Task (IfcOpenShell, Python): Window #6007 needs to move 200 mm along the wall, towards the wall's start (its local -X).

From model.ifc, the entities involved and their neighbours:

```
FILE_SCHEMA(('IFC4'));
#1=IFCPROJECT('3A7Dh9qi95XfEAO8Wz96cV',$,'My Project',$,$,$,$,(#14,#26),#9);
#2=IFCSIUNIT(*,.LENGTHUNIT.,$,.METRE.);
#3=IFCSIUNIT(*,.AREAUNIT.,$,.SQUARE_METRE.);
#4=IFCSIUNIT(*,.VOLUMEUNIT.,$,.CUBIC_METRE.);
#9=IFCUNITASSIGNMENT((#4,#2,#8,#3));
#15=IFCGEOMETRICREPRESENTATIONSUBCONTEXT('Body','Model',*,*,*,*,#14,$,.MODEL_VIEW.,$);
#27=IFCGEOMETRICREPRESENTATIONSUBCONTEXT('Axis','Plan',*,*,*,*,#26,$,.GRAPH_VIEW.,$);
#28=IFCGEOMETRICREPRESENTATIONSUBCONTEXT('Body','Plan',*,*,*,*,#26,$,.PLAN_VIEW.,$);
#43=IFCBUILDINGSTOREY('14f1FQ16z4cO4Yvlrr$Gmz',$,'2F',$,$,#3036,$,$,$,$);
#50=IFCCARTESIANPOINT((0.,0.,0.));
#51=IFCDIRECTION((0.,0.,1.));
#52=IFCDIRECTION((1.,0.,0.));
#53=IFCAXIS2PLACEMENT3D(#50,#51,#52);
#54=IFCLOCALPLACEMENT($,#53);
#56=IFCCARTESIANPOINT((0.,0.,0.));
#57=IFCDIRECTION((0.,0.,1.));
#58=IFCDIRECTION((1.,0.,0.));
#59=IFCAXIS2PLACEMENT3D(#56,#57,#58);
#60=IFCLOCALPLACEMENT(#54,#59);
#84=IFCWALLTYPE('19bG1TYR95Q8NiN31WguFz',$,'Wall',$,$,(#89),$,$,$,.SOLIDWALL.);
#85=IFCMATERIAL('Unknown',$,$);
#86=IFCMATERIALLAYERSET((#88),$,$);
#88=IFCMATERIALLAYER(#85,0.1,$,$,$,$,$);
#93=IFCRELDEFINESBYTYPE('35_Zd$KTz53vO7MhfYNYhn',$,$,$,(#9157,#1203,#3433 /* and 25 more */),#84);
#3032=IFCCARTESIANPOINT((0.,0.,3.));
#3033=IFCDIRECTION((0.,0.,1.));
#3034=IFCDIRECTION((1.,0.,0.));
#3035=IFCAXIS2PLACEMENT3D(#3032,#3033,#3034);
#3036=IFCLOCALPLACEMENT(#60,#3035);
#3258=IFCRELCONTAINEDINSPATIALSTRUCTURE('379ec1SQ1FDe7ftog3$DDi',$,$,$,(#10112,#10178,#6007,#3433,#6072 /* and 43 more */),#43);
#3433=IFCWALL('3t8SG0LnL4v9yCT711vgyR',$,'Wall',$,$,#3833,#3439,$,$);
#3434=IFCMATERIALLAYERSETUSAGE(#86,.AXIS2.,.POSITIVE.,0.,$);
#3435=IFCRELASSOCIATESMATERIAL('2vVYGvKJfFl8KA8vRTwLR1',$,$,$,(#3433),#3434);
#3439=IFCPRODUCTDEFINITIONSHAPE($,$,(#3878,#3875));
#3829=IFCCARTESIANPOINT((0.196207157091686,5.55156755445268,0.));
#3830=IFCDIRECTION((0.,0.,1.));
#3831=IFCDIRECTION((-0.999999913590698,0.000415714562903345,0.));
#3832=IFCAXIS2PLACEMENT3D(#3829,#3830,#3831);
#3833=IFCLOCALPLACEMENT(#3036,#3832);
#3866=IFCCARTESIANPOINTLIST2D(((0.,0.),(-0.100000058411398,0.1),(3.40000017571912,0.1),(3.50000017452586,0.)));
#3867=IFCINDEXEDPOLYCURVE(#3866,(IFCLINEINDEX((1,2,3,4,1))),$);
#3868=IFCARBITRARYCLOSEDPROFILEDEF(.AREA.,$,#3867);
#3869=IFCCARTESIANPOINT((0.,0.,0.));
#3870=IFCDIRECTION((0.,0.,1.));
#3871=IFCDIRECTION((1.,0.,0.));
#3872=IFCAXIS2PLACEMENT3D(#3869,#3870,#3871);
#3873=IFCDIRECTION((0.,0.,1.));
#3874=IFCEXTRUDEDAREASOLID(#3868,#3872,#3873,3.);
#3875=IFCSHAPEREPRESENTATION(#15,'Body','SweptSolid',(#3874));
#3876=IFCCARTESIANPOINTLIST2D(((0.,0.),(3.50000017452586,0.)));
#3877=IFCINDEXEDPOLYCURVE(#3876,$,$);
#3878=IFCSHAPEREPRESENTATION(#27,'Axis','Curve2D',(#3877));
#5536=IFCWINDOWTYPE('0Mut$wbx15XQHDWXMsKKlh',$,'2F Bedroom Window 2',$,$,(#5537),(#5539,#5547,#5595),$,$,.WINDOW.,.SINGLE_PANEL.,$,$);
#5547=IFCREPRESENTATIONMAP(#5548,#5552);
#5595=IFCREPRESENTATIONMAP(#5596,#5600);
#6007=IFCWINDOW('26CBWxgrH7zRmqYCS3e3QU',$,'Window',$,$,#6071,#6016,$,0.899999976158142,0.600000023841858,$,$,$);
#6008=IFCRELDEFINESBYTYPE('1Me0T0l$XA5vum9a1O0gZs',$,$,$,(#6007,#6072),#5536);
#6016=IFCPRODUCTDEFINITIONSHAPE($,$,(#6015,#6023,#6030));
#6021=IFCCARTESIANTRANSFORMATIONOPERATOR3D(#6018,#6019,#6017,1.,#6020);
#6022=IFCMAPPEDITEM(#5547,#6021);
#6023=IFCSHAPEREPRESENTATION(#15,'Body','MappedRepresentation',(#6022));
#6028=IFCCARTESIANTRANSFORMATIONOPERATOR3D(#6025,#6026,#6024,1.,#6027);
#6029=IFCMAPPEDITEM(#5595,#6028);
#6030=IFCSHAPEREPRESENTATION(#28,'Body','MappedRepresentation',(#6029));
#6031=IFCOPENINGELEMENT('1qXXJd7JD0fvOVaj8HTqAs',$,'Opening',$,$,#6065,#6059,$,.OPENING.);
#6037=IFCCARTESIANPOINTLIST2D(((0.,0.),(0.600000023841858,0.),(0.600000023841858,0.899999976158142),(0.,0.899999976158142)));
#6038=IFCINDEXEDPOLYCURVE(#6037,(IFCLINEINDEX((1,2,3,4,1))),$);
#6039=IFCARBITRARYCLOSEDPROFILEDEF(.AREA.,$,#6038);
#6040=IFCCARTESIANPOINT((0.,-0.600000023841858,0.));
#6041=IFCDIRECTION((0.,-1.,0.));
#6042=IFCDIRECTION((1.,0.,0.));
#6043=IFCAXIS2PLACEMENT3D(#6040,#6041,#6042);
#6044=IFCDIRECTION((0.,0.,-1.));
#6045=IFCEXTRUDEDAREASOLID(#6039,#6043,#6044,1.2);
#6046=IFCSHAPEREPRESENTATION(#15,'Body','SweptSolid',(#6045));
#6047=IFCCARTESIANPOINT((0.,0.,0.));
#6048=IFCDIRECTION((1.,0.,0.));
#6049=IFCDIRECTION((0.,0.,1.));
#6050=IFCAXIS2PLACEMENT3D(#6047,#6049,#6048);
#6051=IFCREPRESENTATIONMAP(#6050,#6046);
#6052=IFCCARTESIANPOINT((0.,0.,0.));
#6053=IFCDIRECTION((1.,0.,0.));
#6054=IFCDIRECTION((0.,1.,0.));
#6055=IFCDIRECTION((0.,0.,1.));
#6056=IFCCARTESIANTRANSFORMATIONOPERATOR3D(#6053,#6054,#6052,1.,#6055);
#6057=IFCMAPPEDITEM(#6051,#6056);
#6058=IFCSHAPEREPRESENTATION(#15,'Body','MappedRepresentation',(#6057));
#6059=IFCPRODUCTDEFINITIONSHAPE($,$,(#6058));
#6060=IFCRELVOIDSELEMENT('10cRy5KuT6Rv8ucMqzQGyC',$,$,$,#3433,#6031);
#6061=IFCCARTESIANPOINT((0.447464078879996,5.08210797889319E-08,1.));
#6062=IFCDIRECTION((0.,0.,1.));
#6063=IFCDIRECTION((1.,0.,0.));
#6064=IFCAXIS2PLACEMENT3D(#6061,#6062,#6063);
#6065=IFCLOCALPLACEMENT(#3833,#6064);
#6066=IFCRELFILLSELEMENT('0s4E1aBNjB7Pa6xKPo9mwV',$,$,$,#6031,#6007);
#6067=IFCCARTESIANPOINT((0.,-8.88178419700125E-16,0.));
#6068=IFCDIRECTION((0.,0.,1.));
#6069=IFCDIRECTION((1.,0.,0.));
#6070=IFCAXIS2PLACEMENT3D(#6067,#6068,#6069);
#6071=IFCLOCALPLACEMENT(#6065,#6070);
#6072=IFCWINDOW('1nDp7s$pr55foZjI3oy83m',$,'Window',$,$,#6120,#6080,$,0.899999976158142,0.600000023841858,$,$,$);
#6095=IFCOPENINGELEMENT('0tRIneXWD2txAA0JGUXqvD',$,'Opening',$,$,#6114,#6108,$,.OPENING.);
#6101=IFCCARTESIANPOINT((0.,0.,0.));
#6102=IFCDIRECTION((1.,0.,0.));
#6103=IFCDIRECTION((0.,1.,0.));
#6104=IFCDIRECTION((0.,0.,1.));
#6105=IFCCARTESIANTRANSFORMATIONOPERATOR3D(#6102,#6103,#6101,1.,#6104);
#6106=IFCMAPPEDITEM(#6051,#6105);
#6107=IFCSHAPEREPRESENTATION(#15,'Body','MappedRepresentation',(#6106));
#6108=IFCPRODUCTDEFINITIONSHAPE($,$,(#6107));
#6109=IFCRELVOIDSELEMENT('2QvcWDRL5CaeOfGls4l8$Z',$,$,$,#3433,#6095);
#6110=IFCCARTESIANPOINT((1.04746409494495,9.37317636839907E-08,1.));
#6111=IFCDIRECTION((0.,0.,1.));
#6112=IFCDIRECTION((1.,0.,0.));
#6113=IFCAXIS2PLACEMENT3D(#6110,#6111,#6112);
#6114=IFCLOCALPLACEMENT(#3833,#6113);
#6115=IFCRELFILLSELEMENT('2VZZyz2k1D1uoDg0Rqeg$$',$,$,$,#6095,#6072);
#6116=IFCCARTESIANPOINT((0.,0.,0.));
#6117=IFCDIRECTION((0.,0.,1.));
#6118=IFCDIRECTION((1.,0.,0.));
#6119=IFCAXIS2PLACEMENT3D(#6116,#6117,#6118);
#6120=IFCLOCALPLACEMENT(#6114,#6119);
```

```python
import ifcopenshell
import ifcopenshell.api.geometry
import ifcopenshell.util.placement

model = ifcopenshell.open("model.ifc")

window = model.by_id(6007)
opening = window.FillsVoids[0].RelatingOpeningElement
wall = opening.VoidsElements[0].RelatingBuildingElement

wall_matrix = ifcopenshell.util.placement.get_local_placement(wall.ObjectPlacement)
shift = wall_matrix[:3, 0] * -0.2
before = ifcopenshell.util.placement.get_local_placement(window.ObjectPlacement)[:3, 3].copy()

# The window is placed relative to its opening, so it follows when the opening moves.
matrix = ifcopenshell.util.placement.get_local_placement(opening.ObjectPlacement)
matrix[:3, 3] += shift
ifcopenshell.api.geometry.edit_object_placement(
    model, product=opening, matrix=matrix, is_si=False, should_transform_children=True
)

after = ifcopenshell.util.placement.get_local_placement(window.ObjectPlacement)[:3, 3]
print("window moved by", (after - before).round(3) + 0.0)

model.write("model_edited.ifc")
```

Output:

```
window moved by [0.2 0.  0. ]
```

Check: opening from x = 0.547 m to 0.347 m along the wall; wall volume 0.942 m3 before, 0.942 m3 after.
